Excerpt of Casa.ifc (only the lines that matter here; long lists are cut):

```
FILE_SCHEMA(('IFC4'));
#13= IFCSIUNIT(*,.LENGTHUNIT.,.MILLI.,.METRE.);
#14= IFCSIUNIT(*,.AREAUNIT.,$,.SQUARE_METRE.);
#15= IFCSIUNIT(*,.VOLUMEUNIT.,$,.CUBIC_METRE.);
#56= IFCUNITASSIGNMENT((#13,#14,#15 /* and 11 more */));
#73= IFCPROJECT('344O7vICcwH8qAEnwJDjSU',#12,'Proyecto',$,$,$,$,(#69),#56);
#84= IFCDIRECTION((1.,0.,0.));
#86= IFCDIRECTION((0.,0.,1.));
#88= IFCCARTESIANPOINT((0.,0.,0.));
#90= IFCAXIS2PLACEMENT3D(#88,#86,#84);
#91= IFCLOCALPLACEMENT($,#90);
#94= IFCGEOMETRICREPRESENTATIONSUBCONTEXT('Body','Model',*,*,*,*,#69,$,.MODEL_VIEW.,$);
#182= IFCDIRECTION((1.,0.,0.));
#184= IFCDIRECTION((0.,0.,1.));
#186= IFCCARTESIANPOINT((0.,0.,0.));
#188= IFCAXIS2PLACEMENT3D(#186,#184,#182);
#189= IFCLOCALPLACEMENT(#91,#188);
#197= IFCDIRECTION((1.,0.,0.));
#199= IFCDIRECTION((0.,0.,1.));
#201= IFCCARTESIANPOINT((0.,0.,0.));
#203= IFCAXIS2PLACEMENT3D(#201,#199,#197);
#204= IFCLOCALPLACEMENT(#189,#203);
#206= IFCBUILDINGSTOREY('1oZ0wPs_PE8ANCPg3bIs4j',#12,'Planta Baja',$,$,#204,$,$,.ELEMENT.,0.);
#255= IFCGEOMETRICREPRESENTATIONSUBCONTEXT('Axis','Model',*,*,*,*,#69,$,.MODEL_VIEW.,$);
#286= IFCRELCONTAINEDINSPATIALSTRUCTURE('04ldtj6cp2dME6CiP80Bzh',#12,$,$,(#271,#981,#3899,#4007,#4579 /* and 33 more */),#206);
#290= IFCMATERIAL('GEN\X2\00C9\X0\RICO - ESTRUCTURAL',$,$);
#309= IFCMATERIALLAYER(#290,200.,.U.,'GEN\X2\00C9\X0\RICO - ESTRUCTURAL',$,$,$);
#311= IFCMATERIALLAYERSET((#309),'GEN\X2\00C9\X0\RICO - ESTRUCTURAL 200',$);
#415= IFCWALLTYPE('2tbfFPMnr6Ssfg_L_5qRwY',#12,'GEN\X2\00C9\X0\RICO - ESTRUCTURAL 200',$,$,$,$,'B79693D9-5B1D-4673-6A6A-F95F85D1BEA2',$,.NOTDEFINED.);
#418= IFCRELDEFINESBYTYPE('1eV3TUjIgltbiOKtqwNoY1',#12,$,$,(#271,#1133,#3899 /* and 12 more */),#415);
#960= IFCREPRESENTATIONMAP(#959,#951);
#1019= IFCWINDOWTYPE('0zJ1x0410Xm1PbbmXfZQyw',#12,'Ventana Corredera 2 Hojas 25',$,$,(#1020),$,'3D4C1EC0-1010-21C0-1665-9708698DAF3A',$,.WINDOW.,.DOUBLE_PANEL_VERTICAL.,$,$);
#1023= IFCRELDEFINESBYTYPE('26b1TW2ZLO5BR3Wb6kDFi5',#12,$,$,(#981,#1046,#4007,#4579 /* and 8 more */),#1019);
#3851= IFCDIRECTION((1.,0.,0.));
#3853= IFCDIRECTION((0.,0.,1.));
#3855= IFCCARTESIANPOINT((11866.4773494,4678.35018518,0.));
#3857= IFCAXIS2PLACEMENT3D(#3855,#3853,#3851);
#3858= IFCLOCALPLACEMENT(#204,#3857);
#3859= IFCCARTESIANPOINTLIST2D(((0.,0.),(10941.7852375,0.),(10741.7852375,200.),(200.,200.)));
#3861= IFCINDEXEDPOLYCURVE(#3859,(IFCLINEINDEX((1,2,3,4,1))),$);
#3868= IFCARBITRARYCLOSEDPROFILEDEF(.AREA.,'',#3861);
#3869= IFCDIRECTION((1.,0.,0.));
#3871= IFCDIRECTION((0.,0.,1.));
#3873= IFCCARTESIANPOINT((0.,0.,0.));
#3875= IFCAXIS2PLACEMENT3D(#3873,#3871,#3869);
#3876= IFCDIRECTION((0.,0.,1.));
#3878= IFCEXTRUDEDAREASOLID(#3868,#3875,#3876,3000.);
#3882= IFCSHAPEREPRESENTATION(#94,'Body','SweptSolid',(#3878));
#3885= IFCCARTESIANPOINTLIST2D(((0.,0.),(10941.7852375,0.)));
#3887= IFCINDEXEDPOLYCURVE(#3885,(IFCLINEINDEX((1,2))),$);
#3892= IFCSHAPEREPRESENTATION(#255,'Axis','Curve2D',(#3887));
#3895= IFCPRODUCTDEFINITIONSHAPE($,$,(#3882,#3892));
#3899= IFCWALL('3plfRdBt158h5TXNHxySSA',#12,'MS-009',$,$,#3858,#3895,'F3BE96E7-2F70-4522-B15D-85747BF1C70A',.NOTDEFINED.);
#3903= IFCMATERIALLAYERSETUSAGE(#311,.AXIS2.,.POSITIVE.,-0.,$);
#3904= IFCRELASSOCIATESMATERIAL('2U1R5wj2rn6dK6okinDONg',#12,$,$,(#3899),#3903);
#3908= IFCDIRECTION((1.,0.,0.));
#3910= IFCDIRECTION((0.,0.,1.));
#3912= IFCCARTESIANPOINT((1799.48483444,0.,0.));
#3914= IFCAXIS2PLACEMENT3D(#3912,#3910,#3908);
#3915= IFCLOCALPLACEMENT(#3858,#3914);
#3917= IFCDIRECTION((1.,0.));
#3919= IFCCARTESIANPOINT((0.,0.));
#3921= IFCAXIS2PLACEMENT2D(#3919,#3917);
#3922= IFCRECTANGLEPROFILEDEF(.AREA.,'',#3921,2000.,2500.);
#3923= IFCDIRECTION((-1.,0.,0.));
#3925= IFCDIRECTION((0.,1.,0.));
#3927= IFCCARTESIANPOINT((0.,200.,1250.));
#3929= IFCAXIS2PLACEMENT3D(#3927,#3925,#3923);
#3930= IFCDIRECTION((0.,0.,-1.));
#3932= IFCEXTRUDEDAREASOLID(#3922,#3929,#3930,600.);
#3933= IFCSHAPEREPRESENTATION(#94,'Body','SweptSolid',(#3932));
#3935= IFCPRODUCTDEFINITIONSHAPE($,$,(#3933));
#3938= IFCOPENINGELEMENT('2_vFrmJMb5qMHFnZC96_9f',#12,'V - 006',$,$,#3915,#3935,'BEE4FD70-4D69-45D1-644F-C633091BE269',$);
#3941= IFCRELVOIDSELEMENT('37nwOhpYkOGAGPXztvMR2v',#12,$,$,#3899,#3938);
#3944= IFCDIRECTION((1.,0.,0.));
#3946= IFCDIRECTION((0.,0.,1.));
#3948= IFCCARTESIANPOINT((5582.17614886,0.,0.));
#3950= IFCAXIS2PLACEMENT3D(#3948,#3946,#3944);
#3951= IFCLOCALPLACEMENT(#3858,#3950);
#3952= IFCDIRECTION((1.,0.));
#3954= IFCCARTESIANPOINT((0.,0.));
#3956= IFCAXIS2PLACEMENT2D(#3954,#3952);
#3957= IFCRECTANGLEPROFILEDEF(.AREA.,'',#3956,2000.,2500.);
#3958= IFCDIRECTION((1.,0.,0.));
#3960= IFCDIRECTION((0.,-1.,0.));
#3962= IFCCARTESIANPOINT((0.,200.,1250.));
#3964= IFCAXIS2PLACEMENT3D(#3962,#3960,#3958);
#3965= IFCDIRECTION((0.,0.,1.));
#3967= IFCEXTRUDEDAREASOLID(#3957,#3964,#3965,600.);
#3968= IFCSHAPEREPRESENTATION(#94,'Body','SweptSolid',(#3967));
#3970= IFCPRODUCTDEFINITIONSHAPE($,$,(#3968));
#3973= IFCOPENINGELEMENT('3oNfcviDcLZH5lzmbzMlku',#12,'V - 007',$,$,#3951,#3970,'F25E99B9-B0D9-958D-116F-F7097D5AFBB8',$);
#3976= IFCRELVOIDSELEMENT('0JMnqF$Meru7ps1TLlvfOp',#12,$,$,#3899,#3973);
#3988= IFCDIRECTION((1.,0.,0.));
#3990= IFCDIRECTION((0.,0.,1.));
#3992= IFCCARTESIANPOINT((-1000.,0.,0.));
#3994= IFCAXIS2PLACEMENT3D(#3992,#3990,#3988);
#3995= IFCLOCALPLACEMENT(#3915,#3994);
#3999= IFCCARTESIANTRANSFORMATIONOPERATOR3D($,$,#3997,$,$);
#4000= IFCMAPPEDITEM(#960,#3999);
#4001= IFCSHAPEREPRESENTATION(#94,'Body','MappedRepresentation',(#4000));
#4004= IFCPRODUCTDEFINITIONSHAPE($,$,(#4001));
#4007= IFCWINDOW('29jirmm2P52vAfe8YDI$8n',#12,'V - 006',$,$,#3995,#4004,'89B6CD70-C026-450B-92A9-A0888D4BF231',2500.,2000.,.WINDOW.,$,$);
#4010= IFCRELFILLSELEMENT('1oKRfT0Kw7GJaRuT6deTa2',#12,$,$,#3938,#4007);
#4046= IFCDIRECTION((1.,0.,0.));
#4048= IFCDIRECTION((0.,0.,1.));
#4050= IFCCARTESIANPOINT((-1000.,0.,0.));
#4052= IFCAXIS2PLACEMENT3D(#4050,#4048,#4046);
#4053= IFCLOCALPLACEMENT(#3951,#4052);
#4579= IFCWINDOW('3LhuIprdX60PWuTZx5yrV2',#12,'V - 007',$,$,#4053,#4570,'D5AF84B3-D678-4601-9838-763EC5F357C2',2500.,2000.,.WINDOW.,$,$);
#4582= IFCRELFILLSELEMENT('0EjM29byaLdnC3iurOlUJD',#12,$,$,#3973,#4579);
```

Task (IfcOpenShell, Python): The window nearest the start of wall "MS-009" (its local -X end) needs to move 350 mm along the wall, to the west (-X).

```python
import ifcopenshell
import ifcopenshell.api.geometry
import ifcopenshell.util.placement

model = ifcopenshell.open("Casa.ifc")

window = model.by_guid("29jirmm2P52vAfe8YDI$8n")
opening = window.FillsVoids[0].RelatingOpeningElement
wall = opening.VoidsElements[0].RelatingBuildingElement

wall_matrix = ifcopenshell.util.placement.get_local_placement(wall.ObjectPlacement)
shift = wall_matrix[:3, 0] * -350.0
before = ifcopenshell.util.placement.get_local_placement(window.ObjectPlacement)[:3, 3].copy()

# The window is placed relative to its opening, so it follows when the opening moves.
matrix = ifcopenshell.util.placement.get_local_placement(opening.ObjectPlacement)
matrix[:3, 3] += shift
ifcopenshell.api.geometry.edit_object_placement(
    model, product=opening, matrix=matrix, is_si=False, should_transform_children=True
)

after = ifcopenshell.util.placement.get_local_placement(window.ObjectPlacement)[:3, 3]
print("window moved by", (after - before).round(3) + 0.0)

model.write("Casa_updated.ifc")
```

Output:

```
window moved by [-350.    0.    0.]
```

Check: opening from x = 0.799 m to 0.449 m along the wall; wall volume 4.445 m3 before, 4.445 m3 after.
